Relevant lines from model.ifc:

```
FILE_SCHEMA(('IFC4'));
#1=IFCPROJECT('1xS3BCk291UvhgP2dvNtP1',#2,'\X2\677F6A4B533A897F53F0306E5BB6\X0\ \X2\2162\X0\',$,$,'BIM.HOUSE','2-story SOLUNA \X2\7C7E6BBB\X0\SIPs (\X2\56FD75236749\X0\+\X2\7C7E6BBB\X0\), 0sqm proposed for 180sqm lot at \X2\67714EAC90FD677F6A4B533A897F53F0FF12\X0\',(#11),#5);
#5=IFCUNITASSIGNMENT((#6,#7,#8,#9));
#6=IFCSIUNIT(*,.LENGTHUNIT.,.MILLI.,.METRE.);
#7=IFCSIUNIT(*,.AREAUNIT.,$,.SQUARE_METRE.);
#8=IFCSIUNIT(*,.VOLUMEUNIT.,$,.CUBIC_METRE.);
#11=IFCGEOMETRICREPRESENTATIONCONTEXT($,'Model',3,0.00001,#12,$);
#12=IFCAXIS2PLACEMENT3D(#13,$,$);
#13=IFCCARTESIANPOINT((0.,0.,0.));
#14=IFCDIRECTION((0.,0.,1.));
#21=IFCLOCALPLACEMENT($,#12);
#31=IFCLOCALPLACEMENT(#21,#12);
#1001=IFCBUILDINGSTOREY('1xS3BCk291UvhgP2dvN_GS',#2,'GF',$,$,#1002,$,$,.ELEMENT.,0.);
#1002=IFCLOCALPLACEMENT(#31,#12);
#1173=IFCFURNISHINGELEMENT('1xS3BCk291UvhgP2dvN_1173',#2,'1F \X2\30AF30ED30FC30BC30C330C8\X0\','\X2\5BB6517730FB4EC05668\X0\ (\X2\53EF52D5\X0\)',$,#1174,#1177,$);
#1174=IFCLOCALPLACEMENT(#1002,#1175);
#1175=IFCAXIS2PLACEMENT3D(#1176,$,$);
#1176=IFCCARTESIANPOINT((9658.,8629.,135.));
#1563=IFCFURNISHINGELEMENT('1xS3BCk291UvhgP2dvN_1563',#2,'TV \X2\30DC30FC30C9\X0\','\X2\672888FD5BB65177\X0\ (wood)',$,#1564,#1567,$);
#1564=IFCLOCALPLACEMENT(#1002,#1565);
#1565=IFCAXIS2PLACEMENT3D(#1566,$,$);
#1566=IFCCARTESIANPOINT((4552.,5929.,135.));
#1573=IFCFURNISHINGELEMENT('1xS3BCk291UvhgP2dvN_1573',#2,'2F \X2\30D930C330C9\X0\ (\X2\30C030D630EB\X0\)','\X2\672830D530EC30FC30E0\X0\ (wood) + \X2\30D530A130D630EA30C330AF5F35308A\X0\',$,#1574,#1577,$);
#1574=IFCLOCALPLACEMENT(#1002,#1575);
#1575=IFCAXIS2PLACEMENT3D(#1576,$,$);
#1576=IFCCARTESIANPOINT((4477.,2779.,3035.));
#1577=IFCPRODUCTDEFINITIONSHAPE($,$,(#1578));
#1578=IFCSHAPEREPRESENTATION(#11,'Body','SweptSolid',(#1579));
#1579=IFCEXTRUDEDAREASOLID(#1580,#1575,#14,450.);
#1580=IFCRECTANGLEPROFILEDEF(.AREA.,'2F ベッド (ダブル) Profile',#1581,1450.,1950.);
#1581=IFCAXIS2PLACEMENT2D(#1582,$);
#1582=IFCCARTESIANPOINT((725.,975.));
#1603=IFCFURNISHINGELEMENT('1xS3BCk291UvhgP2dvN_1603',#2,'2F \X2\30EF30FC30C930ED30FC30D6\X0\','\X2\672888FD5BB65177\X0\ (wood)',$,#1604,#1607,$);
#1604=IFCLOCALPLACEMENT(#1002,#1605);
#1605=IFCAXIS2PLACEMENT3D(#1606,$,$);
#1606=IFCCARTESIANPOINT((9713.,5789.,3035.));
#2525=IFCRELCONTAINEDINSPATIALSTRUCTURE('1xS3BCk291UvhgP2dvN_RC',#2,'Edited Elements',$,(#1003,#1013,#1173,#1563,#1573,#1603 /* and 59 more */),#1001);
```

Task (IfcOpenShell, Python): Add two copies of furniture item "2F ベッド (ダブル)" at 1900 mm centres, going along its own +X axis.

```python
import ifcopenshell
import ifcopenshell.api.geometry
import ifcopenshell.api.root
import ifcopenshell.util.element
import ifcopenshell.util.placement
import ifcopenshell.util.unit

model = ifcopenshell.open("model.ifc")
unit_scale = ifcopenshell.util.unit.calculate_unit_scale(model)


def reuse_history(source, copy):
    """copy_class also copies each property set's owner history, people and application; keep the originals."""
    for rel in copy.IsDefinedBy:
        if rel.is_a("IfcRelDefinesByProperties") and (history := rel.RelatingPropertyDefinition.OwnerHistory):
            rel.RelatingPropertyDefinition.OwnerHistory = source.OwnerHistory
            ifcopenshell.util.element.remove_deep2(model, history)


source = model.by_guid("1xS3BCk291UvhgP2dvN_1573")
base = ifcopenshell.util.placement.get_local_placement(source.ObjectPlacement)
step = base[:3, 0] * 1.9 / unit_scale

for i in range(1, 3):
    copy = ifcopenshell.api.root.copy_class(model, product=source)
    copy.Representation = ifcopenshell.util.element.copy_deep(
        model, source.Representation, exclude=["IfcGeometricRepresentationContext", "IfcRepresentationMap"]
    )
    reuse_history(source, copy)
    matrix = base.copy()
    matrix[:3, 3] += i * step
    print("added at", matrix[:3, 3].round(3) + 0.0)
    ifcopenshell.api.geometry.edit_object_placement(model, product=copy, matrix=matrix, is_si=False)

model.write("model-out.ifc")
```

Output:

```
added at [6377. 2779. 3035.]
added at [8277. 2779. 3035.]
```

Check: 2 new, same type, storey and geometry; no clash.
